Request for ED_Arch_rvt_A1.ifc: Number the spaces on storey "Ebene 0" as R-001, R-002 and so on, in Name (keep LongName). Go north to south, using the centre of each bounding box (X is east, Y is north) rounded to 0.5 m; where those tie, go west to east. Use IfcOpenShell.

First a look at what the model holds.

```python
import ifcopenshell
import ifcopenshell.util.element
import ifcopenshell.util.placement

model = ifcopenshell.open("ED_Arch_rvt_A1.ifc")
print(model.schema)
storey = next(s for s in model.by_type("IfcBuildingStorey") if s.Name == "Ebene 0")
spaces = [e for e in ifcopenshell.util.element.get_decomposition(storey) if e.is_a("IfcSpace")]
for e in sorted(spaces, key=lambda e: e.id()):
    origin = ifcopenshell.util.placement.get_local_placement(e.ObjectPlacement)[:3, 3]
    print(e.id(), e.Name, e.LongName, origin.round(2) + 0.0, sep=" | ")
```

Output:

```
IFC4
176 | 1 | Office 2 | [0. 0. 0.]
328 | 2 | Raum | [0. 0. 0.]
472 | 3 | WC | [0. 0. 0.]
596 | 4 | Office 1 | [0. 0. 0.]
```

```python
import ifcopenshell
import ifcopenshell.geom
import ifcopenshell.util.element
import ifcopenshell.util.shape

model = ifcopenshell.open("ED_Arch_rvt_A1.ifc")
settings = ifcopenshell.geom.settings()
settings.set("use-world-coords", True)


def centre(element):
    shape = ifcopenshell.geom.create_shape(settings, element)
    return ifcopenshell.util.shape.get_bbox_centroid(shape.geometry)


storey = next(s for s in model.by_type("IfcBuildingStorey") if s.Name == "Ebene 0")
spaces = [e for e in ifcopenshell.util.element.get_decomposition(storey) if e.is_a("IfcSpace")]

# Insertion points can sit at a corner or the storey origin, so sort by the geometry (in metres).
centres = {e: centre(e) for e in spaces}
spaces.sort(key=lambda e: (-round(centres[e][1] / 0.5), centres[e][0]))

for i, e in enumerate(spaces, start=1):
    number = f"R-0{i:02d}"
    e.Name = number
    print(e.id(), number)

model.write("ED_Arch_rvt_A1_edited.ifc")
```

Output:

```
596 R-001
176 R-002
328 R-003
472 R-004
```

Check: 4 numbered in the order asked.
